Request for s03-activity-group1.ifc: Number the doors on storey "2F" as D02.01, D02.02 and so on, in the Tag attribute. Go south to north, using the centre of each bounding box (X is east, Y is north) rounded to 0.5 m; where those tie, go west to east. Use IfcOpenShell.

First a look at what the model holds.

```python
import ifcopenshell
import ifcopenshell.util.element
import ifcopenshell.util.placement

model = ifcopenshell.open("s03-activity-group1.ifc")
print(model.schema)
storey = next(s for s in model.by_type("IfcBuildingStorey") if s.Name == "2F")
doors = [e for e in ifcopenshell.util.element.get_decomposition(storey) if e.is_a("IfcDoor")]
for e in sorted(doors, key=lambda e: e.id()):
    origin = ifcopenshell.util.placement.get_local_placement(e.ObjectPlacement)[:3, 3]
    print(e.id(), e.Tag, e.Name, origin.round(2) + 0.0, sep=" | ")
```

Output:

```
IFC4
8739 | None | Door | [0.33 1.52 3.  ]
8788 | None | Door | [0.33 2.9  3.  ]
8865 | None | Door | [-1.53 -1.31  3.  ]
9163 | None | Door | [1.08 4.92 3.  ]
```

```python
import ifcopenshell
import ifcopenshell.geom
import ifcopenshell.util.element
import ifcopenshell.util.shape

model = ifcopenshell.open("s03-activity-group1.ifc")
settings = ifcopenshell.geom.settings()
settings.set("use-world-coords", True)


def centre(element):
    shape = ifcopenshell.geom.create_shape(settings, element)
    return ifcopenshell.util.shape.get_bbox_centroid(shape.geometry)


storey = next(s for s in model.by_type("IfcBuildingStorey") if s.Name == "2F")
doors = [e for e in ifcopenshell.util.element.get_decomposition(storey) if e.is_a("IfcDoor")]

# Insertion points can sit at a corner or the storey origin, so sort by the geometry (in metres).
centres = {e: centre(e) for e in doors}
doors.sort(key=lambda e: (round(centres[e][1] / 0.5), centres[e][0]))

for i, e in enumerate(doors, start=1):
    number = f"D02.{i:02d}"
    e.Tag = number
    print(e.id(), number)

model.write("s03-activity-group1_updated.ifc")
```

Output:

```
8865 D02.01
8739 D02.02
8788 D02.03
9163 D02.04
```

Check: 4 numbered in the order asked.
